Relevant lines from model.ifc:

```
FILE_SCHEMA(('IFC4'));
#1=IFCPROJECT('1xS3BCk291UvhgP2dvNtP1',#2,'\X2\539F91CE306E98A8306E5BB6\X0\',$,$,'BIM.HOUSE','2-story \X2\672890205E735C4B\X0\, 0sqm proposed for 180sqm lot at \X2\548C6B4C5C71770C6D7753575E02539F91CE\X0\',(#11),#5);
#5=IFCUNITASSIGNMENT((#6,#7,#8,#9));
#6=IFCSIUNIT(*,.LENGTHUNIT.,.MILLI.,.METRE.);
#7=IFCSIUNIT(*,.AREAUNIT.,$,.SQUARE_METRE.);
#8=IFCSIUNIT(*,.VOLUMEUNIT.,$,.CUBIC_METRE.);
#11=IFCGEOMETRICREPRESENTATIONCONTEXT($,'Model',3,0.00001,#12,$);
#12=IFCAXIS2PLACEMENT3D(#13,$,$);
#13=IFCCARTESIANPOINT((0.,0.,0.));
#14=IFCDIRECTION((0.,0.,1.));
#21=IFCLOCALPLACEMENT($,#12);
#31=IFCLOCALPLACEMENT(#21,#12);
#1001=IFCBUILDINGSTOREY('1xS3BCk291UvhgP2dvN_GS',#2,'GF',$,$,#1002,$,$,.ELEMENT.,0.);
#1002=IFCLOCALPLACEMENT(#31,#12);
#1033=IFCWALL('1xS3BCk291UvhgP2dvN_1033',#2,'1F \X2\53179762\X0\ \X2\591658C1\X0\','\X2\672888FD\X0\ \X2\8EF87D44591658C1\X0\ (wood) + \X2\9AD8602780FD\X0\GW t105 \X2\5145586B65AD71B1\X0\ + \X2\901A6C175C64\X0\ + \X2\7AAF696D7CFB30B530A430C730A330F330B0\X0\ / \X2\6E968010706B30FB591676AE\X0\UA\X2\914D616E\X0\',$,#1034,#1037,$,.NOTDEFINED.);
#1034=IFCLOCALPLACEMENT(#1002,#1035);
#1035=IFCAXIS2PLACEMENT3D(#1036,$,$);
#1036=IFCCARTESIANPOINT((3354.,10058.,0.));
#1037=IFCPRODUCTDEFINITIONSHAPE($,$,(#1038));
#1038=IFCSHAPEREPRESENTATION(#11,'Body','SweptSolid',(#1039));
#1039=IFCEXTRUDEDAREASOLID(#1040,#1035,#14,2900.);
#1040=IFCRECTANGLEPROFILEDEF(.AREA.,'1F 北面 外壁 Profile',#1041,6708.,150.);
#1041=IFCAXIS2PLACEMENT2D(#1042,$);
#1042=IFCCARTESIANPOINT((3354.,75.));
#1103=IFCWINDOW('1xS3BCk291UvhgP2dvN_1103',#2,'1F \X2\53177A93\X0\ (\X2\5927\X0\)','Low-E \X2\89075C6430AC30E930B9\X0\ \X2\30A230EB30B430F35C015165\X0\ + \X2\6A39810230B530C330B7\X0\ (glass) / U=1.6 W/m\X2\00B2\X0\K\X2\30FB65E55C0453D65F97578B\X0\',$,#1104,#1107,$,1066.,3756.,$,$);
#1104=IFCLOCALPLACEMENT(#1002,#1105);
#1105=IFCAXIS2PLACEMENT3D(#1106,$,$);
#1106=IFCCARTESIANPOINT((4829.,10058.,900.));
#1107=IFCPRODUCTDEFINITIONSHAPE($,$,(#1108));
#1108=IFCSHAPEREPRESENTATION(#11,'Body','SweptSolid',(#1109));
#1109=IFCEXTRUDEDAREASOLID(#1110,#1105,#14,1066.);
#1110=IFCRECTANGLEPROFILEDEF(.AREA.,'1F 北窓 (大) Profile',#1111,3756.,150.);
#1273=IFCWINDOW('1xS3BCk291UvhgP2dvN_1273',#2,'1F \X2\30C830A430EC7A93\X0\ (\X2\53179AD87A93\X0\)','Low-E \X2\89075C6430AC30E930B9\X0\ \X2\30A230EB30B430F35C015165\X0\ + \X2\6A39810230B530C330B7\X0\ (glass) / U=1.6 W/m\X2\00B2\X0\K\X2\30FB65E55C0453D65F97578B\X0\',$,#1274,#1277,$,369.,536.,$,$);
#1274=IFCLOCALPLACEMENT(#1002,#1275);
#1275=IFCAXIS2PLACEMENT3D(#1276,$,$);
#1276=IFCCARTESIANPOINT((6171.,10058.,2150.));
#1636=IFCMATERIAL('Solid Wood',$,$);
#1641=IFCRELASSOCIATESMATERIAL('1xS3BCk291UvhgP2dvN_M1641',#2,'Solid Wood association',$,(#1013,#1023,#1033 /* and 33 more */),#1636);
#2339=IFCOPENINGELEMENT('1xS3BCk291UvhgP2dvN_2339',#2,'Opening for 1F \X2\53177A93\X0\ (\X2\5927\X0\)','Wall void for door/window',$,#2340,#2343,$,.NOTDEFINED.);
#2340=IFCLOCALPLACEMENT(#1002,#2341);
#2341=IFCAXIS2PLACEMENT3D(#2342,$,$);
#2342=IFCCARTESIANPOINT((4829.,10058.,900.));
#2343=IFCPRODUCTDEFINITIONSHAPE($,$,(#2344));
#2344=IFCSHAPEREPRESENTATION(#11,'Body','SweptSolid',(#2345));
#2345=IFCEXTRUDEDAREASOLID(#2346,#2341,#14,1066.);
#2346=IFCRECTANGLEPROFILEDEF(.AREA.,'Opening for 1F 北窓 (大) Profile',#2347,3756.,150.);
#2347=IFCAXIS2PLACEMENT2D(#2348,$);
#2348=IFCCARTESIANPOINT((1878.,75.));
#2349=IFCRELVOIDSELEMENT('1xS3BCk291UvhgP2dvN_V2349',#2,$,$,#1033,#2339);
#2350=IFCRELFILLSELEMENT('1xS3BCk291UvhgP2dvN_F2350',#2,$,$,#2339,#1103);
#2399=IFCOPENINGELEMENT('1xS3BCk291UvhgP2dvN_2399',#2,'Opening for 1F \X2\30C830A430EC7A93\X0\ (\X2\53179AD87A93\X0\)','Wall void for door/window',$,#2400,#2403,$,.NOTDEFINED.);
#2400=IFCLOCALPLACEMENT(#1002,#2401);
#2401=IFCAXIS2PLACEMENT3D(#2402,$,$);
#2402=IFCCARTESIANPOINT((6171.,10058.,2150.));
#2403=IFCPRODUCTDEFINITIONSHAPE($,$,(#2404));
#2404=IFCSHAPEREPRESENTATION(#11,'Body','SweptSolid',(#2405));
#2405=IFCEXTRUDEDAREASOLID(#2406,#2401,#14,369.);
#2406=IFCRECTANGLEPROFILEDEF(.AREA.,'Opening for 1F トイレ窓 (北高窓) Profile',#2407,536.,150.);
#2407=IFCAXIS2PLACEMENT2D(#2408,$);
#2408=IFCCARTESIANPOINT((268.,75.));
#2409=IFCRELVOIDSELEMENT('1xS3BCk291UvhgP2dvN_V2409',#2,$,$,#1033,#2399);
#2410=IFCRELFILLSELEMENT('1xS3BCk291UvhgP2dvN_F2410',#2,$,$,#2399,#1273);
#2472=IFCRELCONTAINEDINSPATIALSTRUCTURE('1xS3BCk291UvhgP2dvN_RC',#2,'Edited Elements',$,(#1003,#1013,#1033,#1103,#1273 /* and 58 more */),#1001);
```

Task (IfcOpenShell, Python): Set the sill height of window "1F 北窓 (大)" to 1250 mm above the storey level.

```python
import numpy as np
import ifcopenshell
import ifcopenshell.api.geometry
import ifcopenshell.geom
import ifcopenshell.util.element
import ifcopenshell.util.placement
import ifcopenshell.util.shape
import ifcopenshell.util.unit

model = ifcopenshell.open("model.ifc")
unit_scale = ifcopenshell.util.unit.calculate_unit_scale(model)

window = model.by_guid("1xS3BCk291UvhgP2dvN_1103")
opening = window.FillsVoids[0].RelatingOpeningElement
storey = ifcopenshell.util.element.get_container(window, ifc_class="IfcBuildingStorey")
level = ifcopenshell.util.placement.get_local_placement(storey.ObjectPlacement)[2, 3]

# The opening's origin need not be at the sill, so measure its lowest point.
shape = ifcopenshell.geom.create_shape(ifcopenshell.geom.settings(), opening)
bottom = ifcopenshell.util.shape.get_shape_bottom_elevation(shape, shape.geometry) / unit_scale
dz = level + 1250.0 - bottom

shift = np.array([0.0, 0.0, dz])
# The window is not placed relative to its opening, so move both.
for product in (opening, window):
    matrix = ifcopenshell.util.placement.get_local_placement(product.ObjectPlacement)
    matrix[:3, 3] += shift
    ifcopenshell.api.geometry.edit_object_placement(model, product=product, matrix=matrix, is_si=False)

print(f"moved by {dz * unit_scale:+.3f} m")

model.write("model_updated.ifc")
```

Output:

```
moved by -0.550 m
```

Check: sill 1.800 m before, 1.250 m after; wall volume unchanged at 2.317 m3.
